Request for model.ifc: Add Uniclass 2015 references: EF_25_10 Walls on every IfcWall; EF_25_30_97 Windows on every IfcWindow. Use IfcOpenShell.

First a look at what the model holds.

```python
import ifcopenshell

model = ifcopenshell.open("model.ifc")
print(model.schema)
print("classifications:", [c.Name for c in model.by_type("IfcClassification")])
for ifc_class in ("IfcDoor", "IfcRoof", "IfcStair", "IfcWall", "IfcWindow"):
    print(ifc_class, len(model.by_type(ifc_class)))
```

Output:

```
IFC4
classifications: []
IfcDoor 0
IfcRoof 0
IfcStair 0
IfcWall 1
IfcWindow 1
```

```python
import ifcopenshell
import ifcopenshell.api.classification

model = ifcopenshell.open("model.ifc")

system = ifcopenshell.api.classification.add_classification(model, classification="Uniclass 2015")

codes = {
    "IfcWall": ("EF_25_10", "Walls"),
    "IfcWindow": ("EF_25_30_97", "Windows"),
}
for ifc_class, (code, name) in codes.items():
    products = model.by_type(ifc_class)
    ifcopenshell.api.classification.add_reference(
        model, products=products, classification=system, identification=code, name=name
    )
    print(code, len(products))

model.write("model_v2.ifc")
```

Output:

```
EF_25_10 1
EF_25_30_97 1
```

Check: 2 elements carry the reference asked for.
